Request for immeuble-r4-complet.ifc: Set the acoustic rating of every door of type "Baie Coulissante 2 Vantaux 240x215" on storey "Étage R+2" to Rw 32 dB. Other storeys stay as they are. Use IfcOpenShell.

First a look at what the model holds.

```python
import ifcopenshell
import ifcopenshell.util.element

model = ifcopenshell.open("immeuble-r4-complet.ifc")
print(model.schema)
storey = next(s for s in model.by_type("IfcBuildingStorey") if s.Name == "Étage R+2")
doors = [e for e in ifcopenshell.util.element.get_decomposition(storey) if e.is_a("IfcDoor")]
seen = {}
for e in doors:
    element_type = ifcopenshell.util.element.get_type(e)
    key = (element_type.Name if element_type != e and element_type else None, ifcopenshell.util.element.get_pset(e, "Pset_DoorCommon", "AcousticRating"))
    seen[key] = seen.get(key, 0) + 1
for (name, value), count in sorted(seen.items(), key=str):
    print(count, "x", name, "|", value)
```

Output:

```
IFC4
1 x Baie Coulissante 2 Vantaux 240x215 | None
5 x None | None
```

```python
import ifcopenshell
import ifcopenshell.api.pset
import ifcopenshell.util.element

model = ifcopenshell.open("immeuble-r4-complet.ifc")

storey = next(s for s in model.by_type("IfcBuildingStorey") if s.Name == "Étage R+2")
doors = [e for e in ifcopenshell.util.element.get_decomposition(storey) if e.is_a("IfcDoor")]

count = 0
for e in doors:
    element_type = ifcopenshell.util.element.get_type(e)
    if element_type in (None, e) or element_type.Name != "Baie Coulissante 2 Vantaux 240x215":
        continue
    # add_pset returns the element's existing set when there is one.
    pset = ifcopenshell.api.pset.add_pset(model, product=e, name="Pset_DoorCommon")
    ifcopenshell.api.pset.edit_pset(model, pset=pset, properties={"AcousticRating": "Rw 32 dB"})
    count += 1

print(count, "doors updated")

model.write("immeuble-r4-complet_updated.ifc")
```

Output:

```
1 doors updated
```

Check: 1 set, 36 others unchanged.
